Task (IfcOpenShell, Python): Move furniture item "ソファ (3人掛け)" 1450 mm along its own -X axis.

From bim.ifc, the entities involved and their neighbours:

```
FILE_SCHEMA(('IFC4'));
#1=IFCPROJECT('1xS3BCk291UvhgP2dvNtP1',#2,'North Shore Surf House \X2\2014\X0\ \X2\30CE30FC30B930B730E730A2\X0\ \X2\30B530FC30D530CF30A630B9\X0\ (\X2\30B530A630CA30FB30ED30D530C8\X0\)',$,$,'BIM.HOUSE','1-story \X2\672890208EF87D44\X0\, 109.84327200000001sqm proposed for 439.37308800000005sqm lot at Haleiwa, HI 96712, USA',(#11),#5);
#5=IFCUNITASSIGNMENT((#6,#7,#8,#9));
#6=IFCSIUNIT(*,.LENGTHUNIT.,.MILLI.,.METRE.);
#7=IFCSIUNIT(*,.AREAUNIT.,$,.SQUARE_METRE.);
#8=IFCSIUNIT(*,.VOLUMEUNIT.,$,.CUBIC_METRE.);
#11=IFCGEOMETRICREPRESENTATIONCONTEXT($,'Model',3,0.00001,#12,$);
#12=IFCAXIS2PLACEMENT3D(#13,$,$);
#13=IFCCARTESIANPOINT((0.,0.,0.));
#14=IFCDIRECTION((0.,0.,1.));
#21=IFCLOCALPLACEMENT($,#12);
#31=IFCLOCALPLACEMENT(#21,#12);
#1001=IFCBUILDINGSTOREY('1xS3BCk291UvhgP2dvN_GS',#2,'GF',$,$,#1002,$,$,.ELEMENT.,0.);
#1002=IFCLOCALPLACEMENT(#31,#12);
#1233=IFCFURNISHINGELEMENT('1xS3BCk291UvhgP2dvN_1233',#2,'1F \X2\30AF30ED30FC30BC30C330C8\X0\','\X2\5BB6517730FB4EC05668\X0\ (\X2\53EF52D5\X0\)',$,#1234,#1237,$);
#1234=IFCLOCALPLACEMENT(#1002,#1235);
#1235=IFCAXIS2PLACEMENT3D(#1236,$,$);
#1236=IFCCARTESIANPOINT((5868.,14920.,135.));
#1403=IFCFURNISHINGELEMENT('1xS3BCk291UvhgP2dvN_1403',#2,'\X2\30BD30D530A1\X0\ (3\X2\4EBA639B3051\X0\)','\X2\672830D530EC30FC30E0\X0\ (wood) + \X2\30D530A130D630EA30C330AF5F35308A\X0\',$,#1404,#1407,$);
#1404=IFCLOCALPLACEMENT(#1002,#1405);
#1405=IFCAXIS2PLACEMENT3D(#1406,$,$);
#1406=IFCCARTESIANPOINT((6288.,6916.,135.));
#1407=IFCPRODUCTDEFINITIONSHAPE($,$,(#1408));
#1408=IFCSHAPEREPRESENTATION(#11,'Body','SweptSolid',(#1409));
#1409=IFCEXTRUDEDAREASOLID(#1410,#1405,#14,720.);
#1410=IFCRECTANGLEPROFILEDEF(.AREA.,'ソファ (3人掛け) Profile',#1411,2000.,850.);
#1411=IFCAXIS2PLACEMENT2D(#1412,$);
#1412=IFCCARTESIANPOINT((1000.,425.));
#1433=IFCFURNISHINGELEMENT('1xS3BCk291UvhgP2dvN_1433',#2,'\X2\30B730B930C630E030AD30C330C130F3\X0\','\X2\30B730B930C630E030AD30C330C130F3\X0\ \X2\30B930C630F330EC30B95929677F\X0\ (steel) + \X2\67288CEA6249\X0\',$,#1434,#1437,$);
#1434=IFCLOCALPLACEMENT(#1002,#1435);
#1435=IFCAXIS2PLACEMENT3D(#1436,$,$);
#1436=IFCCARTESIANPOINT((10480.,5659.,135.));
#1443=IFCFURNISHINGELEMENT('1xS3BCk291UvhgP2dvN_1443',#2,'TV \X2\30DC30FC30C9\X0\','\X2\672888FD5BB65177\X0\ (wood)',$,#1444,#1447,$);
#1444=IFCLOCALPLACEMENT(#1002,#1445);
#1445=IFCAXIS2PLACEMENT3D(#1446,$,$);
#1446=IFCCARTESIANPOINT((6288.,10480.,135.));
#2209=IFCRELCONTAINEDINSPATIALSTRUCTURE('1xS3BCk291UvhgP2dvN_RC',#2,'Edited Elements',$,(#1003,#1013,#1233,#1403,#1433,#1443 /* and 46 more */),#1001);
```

```python
import ifcopenshell
import ifcopenshell.api.geometry
import ifcopenshell.util.placement
import ifcopenshell.util.unit

model = ifcopenshell.open("bim.ifc")
unit_scale = ifcopenshell.util.unit.calculate_unit_scale(model)

item = model.by_guid("1xS3BCk291UvhgP2dvN_1403")
matrix = ifcopenshell.util.placement.get_local_placement(item.ObjectPlacement)
matrix[:3, 3] -= matrix[:3, 0] * 1.45 / unit_scale
ifcopenshell.api.geometry.edit_object_placement(model, product=item, matrix=matrix, is_si=False)

print(ifcopenshell.util.placement.get_local_placement(item.ObjectPlacement).round(3) + 0.0)

model.write("bim_v2.ifc")
```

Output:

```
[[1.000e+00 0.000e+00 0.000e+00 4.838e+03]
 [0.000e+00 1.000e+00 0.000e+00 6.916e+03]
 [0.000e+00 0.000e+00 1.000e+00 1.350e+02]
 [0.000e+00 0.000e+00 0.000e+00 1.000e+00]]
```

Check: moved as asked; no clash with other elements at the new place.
